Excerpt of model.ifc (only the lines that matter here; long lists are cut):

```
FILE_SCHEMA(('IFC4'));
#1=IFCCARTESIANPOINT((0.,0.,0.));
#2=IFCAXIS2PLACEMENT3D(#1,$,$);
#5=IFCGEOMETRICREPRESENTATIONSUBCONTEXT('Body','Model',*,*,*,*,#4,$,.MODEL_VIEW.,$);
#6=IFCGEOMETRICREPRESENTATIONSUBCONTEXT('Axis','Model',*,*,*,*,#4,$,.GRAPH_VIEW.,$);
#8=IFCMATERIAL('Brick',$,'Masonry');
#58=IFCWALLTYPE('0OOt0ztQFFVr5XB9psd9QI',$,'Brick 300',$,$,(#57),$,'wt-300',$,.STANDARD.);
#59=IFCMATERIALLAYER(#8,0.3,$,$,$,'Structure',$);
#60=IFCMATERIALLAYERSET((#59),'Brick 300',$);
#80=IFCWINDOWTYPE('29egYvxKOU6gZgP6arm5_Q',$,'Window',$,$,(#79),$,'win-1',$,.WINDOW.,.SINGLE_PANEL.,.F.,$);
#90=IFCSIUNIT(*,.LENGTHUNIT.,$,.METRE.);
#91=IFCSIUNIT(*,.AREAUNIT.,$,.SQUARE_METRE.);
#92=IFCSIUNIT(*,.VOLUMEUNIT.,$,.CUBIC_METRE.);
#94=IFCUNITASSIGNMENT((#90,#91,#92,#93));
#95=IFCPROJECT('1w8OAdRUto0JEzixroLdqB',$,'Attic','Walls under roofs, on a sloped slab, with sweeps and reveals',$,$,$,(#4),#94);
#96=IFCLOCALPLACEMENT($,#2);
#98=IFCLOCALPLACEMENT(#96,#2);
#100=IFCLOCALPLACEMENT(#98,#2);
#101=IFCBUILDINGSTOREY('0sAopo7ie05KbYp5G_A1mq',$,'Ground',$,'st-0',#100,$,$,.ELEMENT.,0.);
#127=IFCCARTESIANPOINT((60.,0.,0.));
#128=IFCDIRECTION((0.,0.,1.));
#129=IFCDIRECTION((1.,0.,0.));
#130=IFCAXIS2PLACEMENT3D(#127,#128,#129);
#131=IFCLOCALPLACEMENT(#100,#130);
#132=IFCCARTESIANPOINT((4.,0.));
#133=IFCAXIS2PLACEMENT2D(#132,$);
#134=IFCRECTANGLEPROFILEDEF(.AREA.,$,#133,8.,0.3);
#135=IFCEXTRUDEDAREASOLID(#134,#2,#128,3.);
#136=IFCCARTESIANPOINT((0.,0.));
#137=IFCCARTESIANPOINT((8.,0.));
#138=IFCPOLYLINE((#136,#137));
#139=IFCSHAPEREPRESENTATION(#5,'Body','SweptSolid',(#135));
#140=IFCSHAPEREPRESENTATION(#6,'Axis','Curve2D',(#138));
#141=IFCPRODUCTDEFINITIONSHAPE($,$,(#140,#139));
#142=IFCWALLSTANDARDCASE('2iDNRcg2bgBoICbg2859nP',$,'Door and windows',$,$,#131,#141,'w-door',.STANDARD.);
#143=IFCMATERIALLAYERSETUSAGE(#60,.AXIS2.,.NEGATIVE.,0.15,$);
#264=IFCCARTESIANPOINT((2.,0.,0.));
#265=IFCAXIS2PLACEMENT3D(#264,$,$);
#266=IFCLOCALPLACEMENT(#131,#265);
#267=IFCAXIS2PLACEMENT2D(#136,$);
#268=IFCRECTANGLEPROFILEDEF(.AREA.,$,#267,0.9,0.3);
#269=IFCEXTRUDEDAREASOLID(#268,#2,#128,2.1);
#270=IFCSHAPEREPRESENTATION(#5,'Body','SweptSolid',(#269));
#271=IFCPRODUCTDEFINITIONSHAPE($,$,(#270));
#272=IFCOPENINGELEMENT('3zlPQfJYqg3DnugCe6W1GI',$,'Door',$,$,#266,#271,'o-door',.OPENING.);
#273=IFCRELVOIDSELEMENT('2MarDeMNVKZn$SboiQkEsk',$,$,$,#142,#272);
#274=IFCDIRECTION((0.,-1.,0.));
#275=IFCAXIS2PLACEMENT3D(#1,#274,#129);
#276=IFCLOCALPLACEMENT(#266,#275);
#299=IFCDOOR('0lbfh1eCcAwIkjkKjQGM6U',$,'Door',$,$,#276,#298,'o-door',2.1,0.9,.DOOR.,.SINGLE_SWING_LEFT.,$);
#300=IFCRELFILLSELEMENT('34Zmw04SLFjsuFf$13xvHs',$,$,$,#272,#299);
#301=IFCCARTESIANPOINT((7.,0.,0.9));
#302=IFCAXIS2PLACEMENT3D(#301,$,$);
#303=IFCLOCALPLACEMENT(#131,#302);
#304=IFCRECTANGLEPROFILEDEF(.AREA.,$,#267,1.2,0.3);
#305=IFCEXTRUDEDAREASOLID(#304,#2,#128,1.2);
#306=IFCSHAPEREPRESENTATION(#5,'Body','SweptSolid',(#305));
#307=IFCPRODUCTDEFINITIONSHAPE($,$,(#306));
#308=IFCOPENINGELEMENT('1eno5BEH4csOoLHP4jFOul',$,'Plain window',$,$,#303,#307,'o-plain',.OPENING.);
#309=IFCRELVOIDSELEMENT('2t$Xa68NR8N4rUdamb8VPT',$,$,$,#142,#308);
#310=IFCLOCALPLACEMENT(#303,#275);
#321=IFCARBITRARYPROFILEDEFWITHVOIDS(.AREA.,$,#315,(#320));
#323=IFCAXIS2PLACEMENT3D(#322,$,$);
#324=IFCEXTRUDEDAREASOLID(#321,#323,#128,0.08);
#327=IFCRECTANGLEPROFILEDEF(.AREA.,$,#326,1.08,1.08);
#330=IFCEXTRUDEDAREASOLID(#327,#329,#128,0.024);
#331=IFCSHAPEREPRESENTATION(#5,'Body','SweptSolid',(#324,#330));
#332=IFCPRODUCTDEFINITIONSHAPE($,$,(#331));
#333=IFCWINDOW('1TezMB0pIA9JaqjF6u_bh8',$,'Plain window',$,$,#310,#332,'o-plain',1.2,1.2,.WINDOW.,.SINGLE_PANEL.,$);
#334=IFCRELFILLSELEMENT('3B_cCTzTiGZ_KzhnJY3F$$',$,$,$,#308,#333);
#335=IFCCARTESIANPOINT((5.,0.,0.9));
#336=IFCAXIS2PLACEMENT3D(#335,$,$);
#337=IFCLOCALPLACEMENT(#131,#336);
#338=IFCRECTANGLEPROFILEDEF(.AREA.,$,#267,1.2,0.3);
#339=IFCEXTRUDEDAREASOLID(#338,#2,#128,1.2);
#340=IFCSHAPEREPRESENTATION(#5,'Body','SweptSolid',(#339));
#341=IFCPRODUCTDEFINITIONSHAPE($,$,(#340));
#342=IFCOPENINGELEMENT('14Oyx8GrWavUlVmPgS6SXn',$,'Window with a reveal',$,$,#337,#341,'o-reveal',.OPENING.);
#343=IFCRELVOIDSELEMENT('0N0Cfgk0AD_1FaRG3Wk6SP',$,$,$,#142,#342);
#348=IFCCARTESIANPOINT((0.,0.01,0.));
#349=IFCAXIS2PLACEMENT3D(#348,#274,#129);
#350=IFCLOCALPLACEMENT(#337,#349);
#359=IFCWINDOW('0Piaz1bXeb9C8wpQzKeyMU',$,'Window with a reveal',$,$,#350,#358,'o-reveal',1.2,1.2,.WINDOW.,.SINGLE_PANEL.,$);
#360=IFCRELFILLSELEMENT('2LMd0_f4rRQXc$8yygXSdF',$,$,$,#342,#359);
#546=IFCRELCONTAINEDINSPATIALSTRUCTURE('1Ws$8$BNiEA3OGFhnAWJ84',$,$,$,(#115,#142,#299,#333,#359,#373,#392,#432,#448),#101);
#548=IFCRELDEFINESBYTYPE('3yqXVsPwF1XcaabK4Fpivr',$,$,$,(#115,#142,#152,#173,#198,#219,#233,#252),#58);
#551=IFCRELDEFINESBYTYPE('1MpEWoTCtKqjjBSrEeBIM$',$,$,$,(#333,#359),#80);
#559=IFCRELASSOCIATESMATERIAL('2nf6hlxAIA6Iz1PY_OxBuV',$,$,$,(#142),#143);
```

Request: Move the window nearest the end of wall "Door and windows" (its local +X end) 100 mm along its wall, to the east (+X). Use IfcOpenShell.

```python
import ifcopenshell
import ifcopenshell.api.geometry
import ifcopenshell.util.placement

model = ifcopenshell.open("model.ifc")

window = model.by_guid("1TezMB0pIA9JaqjF6u_bh8")
opening = window.FillsVoids[0].RelatingOpeningElement
wall = opening.VoidsElements[0].RelatingBuildingElement

wall_matrix = ifcopenshell.util.placement.get_local_placement(wall.ObjectPlacement)
shift = wall_matrix[:3, 0] * 0.1
before = ifcopenshell.util.placement.get_local_placement(window.ObjectPlacement)[:3, 3].copy()

# The window is placed relative to its opening, so it follows when the opening moves.
matrix = ifcopenshell.util.placement.get_local_placement(opening.ObjectPlacement)
matrix[:3, 3] += shift
ifcopenshell.api.geometry.edit_object_placement(
    model, product=opening, matrix=matrix, is_si=False, should_transform_children=True
)

after = ifcopenshell.util.placement.get_local_placement(window.ObjectPlacement)[:3, 3]
print("window moved by", (after - before).round(3) + 0.0)

model.write("model_rev.ifc")
```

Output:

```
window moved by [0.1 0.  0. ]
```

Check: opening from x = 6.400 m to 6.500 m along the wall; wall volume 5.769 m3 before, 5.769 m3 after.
